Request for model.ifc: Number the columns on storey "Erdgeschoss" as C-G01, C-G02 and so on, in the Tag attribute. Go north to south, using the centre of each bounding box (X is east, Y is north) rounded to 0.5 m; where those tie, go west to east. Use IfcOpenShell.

First a look at what the model holds.

```python
import ifcopenshell
import ifcopenshell.util.element
import ifcopenshell.util.placement

model = ifcopenshell.open("model.ifc")
print(model.schema)
storey = next(s for s in model.by_type("IfcBuildingStorey") if s.Name == "Erdgeschoss")
columns = [e for e in ifcopenshell.util.element.get_decomposition(storey) if e.is_a("IfcColumn")]
for e in sorted(columns, key=lambda e: e.id()):
    origin = ifcopenshell.util.placement.get_local_placement(e.ObjectPlacement)[:3, 3]
    print(e.id(), e.Tag, e.Name, origin.round(2) + 0.0, sep=" | ")
```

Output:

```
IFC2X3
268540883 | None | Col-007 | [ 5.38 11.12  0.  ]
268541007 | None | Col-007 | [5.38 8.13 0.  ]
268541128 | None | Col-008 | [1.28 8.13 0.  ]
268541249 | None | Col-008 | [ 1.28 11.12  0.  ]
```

```python
import ifcopenshell
import ifcopenshell.geom
import ifcopenshell.util.element
import ifcopenshell.util.shape

model = ifcopenshell.open("model.ifc")
settings = ifcopenshell.geom.settings()
settings.set("use-world-coords", True)


def centre(element):
    shape = ifcopenshell.geom.create_shape(settings, element)
    return ifcopenshell.util.shape.get_bbox_centroid(shape.geometry)


storey = next(s for s in model.by_type("IfcBuildingStorey") if s.Name == "Erdgeschoss")
columns = [e for e in ifcopenshell.util.element.get_decomposition(storey) if e.is_a("IfcColumn")]

# Insertion points can sit at a corner or the storey origin, so sort by the geometry (in metres).
centres = {e: centre(e) for e in columns}
columns.sort(key=lambda e: (-round(centres[e][1] / 0.5), centres[e][0]))

for i, e in enumerate(columns, start=1):
    number = f"C-G{i:02d}"
    e.Tag = number
    print(e.id(), number)

model.write("model_rev.ifc")
```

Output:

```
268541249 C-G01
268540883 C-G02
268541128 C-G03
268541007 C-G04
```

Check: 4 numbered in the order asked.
